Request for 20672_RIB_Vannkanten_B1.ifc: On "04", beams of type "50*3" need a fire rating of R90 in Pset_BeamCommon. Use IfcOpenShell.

First a look at what the model holds.

```python
import ifcopenshell
import ifcopenshell.util.element

model = ifcopenshell.open("20672_RIB_Vannkanten_B1.ifc")
print(model.schema)
storey = next(s for s in model.by_type("IfcBuildingStorey") if s.Name == "04")
beams = [e for e in ifcopenshell.util.element.get_decomposition(storey) if e.is_a("IfcBeam")]
seen = {}
for e in beams:
    element_type = ifcopenshell.util.element.get_type(e)
    key = (element_type.Name if element_type != e and element_type else None, ifcopenshell.util.element.get_pset(e, "Pset_BeamCommon", "FireRating"))
    seen[key] = seen.get(key, 0) + 1
for (name, value), count in sorted(seen.items(), key=str):
    print(count, "x", name, "|", value)
```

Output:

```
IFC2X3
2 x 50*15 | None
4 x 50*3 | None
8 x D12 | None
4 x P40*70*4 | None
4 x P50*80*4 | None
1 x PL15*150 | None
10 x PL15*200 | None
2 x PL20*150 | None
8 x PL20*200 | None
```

```python
import ifcopenshell
import ifcopenshell.api.pset
import ifcopenshell.util.element

model = ifcopenshell.open("20672_RIB_Vannkanten_B1.ifc")

storey = next(s for s in model.by_type("IfcBuildingStorey") if s.Name == "04")
beams = [e for e in ifcopenshell.util.element.get_decomposition(storey) if e.is_a("IfcBeam")]

count = 0
for e in beams:
    element_type = ifcopenshell.util.element.get_type(e)
    if element_type in (None, e) or element_type.Name != "50*3":
        continue
    # add_pset returns the element's existing set when there is one.
    pset = ifcopenshell.api.pset.add_pset(model, product=e, name="Pset_BeamCommon")
    ifcopenshell.api.pset.edit_pset(model, pset=pset, properties={"FireRating": "R90"})
    count += 1

print(count, "beams updated")

model.write("20672_RIB_Vannkanten_B1_updated.ifc")
```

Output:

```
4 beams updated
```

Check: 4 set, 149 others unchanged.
